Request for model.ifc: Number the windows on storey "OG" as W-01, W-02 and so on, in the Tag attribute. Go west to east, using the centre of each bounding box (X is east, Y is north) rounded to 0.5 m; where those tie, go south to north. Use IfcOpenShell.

First a look at what the model holds.

```python
import ifcopenshell
import ifcopenshell.util.element
import ifcopenshell.util.placement

model = ifcopenshell.open("model.ifc")
print(model.schema)
storey = next(s for s in model.by_type("IfcBuildingStorey") if s.Name == "OG")
windows = [e for e in ifcopenshell.util.element.get_decomposition(storey) if e.is_a("IfcWindow")]
for e in sorted(windows, key=lambda e: e.id()):
    origin = ifcopenshell.util.placement.get_local_placement(e.ObjectPlacement)[:3, 3]
    print(e.id(), e.Tag, e.Name, origin.round(2) + 0.0, sep=" | ")
```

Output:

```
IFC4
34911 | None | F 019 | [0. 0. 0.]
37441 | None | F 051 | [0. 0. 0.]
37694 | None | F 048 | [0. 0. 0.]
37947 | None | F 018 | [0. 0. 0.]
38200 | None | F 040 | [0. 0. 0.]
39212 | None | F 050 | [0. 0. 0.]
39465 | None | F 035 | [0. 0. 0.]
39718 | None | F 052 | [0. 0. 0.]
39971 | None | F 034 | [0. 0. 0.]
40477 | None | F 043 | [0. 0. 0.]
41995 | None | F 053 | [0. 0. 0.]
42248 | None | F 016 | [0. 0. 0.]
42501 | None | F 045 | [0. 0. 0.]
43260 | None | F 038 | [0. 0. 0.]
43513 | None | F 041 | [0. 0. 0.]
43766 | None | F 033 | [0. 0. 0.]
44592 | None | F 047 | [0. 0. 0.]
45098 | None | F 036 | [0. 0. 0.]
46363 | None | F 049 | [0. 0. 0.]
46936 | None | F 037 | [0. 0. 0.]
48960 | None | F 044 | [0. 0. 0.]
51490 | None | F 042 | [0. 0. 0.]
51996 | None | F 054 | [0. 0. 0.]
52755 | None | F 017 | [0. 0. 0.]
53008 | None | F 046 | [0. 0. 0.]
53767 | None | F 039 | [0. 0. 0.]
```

```python
import ifcopenshell
import ifcopenshell.geom
import ifcopenshell.util.element
import ifcopenshell.util.shape

model = ifcopenshell.open("model.ifc")
settings = ifcopenshell.geom.settings()
settings.set("use-world-coords", True)


def centre(element):
    shape = ifcopenshell.geom.create_shape(settings, element)
    return ifcopenshell.util.shape.get_bbox_centroid(shape.geometry)


storey = next(s for s in model.by_type("IfcBuildingStorey") if s.Name == "OG")
windows = [e for e in ifcopenshell.util.element.get_decomposition(storey) if e.is_a("IfcWindow")]

# Insertion points can sit at a corner or the storey origin, so sort by the geometry (in metres).
centres = {e: centre(e) for e in windows}
windows.sort(key=lambda e: (round(centres[e][0] / 0.5), centres[e][1]))

for i, e in enumerate(windows, start=1):
    number = f"W-{i:02d}"
    e.Tag = number
    print(e.id(), number)

model.write("model_updated.ifc")
```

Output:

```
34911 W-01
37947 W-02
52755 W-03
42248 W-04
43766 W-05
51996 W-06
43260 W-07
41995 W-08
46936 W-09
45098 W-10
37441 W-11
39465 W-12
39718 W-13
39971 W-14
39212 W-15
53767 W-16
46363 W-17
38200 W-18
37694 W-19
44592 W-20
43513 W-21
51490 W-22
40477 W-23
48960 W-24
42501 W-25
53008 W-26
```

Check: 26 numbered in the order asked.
